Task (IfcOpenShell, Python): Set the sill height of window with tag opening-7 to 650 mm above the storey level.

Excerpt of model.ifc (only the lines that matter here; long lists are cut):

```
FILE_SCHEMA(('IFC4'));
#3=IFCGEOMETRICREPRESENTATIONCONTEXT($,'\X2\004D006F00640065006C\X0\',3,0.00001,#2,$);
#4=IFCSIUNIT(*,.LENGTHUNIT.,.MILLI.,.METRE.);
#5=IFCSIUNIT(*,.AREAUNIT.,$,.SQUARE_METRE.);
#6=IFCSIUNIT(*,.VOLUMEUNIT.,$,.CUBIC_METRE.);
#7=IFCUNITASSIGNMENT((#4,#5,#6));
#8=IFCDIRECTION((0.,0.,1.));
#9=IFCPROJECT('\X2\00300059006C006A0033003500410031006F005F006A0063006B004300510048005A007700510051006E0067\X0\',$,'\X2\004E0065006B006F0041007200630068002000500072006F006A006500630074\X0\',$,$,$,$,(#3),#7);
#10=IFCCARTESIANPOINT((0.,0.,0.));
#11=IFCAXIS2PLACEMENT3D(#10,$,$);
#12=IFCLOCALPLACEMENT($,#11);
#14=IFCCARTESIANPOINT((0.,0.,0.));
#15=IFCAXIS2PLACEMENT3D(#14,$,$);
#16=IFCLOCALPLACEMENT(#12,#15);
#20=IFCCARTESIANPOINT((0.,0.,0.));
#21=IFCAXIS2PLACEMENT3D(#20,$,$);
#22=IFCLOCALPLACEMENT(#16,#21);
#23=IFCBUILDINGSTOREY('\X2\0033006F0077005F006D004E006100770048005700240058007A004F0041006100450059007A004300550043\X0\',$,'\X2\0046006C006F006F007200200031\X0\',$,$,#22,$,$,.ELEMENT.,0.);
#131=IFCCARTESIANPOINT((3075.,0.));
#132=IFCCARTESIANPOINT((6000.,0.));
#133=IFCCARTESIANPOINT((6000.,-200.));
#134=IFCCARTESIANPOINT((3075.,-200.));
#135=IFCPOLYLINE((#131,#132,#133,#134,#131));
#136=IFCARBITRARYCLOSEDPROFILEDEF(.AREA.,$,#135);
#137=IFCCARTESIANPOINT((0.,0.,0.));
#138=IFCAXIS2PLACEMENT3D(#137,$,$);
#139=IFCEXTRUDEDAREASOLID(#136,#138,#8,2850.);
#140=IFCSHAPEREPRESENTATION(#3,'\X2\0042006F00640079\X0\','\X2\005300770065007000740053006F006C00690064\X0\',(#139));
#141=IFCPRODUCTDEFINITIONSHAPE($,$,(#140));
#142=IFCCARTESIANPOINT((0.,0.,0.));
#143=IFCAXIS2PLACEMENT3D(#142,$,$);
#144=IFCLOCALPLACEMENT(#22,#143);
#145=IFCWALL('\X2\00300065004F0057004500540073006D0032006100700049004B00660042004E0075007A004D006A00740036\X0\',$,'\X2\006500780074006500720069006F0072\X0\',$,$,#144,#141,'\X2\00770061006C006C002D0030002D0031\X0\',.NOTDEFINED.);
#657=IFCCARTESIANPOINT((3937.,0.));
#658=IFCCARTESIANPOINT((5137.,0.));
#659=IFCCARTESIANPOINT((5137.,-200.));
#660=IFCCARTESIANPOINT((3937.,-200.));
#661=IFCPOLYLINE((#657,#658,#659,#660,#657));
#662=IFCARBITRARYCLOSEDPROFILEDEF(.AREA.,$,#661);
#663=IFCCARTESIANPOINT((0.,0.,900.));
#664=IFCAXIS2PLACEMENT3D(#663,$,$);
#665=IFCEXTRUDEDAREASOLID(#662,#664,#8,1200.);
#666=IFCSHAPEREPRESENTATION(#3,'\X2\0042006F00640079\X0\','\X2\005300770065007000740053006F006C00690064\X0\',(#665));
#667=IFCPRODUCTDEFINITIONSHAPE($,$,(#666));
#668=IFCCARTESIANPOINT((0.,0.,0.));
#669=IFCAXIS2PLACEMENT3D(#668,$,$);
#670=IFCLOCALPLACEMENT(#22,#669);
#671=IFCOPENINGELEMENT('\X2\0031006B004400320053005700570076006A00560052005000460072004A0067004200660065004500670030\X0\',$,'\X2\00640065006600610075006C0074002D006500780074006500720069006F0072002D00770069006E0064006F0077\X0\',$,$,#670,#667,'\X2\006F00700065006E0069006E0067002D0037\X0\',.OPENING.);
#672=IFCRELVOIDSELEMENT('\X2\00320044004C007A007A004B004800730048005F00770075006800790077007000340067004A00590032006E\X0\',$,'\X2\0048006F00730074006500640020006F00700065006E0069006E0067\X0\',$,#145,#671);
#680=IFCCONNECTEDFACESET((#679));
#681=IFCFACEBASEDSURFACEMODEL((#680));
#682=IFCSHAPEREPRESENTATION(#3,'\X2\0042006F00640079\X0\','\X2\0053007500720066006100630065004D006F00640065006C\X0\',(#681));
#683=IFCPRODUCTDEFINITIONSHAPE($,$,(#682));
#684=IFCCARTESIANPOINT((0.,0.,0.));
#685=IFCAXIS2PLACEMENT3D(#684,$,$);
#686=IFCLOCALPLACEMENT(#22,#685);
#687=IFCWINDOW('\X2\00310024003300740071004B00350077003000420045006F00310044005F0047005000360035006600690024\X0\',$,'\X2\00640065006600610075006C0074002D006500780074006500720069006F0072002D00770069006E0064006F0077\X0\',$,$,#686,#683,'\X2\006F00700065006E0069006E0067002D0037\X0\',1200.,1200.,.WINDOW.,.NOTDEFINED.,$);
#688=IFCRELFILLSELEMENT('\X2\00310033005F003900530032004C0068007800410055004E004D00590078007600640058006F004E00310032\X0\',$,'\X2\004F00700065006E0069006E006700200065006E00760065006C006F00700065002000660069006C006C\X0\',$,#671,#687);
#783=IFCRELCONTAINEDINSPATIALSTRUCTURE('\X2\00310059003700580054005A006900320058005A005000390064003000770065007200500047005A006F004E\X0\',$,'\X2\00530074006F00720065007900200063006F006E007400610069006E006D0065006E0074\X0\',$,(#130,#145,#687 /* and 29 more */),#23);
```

```python
import numpy as np
import ifcopenshell
import ifcopenshell.api.geometry
import ifcopenshell.geom
import ifcopenshell.util.element
import ifcopenshell.util.placement
import ifcopenshell.util.shape
import ifcopenshell.util.unit

model = ifcopenshell.open("model.ifc")
unit_scale = ifcopenshell.util.unit.calculate_unit_scale(model)

window = model.by_id(687)
opening = window.FillsVoids[0].RelatingOpeningElement
storey = ifcopenshell.util.element.get_container(window, ifc_class="IfcBuildingStorey")
level = ifcopenshell.util.placement.get_local_placement(storey.ObjectPlacement)[2, 3]

# The opening's origin need not be at the sill, so measure its lowest point.
shape = ifcopenshell.geom.create_shape(ifcopenshell.geom.settings(), opening)
bottom = ifcopenshell.util.shape.get_shape_bottom_elevation(shape, shape.geometry) / unit_scale
dz = level + 0.65 / unit_scale - bottom

shift = np.array([0.0, 0.0, dz])
# The window is not placed relative to its opening, so move both.
for product in (opening, window):
    matrix = ifcopenshell.util.placement.get_local_placement(product.ObjectPlacement)
    matrix[:3, 3] += shift
    ifcopenshell.api.geometry.edit_object_placement(model, product=product, matrix=matrix, is_si=False)

print(f"moved by {dz * unit_scale:+.3f} m")

model.write("model_v2.ifc")
```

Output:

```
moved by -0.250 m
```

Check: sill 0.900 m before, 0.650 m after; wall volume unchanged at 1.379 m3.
